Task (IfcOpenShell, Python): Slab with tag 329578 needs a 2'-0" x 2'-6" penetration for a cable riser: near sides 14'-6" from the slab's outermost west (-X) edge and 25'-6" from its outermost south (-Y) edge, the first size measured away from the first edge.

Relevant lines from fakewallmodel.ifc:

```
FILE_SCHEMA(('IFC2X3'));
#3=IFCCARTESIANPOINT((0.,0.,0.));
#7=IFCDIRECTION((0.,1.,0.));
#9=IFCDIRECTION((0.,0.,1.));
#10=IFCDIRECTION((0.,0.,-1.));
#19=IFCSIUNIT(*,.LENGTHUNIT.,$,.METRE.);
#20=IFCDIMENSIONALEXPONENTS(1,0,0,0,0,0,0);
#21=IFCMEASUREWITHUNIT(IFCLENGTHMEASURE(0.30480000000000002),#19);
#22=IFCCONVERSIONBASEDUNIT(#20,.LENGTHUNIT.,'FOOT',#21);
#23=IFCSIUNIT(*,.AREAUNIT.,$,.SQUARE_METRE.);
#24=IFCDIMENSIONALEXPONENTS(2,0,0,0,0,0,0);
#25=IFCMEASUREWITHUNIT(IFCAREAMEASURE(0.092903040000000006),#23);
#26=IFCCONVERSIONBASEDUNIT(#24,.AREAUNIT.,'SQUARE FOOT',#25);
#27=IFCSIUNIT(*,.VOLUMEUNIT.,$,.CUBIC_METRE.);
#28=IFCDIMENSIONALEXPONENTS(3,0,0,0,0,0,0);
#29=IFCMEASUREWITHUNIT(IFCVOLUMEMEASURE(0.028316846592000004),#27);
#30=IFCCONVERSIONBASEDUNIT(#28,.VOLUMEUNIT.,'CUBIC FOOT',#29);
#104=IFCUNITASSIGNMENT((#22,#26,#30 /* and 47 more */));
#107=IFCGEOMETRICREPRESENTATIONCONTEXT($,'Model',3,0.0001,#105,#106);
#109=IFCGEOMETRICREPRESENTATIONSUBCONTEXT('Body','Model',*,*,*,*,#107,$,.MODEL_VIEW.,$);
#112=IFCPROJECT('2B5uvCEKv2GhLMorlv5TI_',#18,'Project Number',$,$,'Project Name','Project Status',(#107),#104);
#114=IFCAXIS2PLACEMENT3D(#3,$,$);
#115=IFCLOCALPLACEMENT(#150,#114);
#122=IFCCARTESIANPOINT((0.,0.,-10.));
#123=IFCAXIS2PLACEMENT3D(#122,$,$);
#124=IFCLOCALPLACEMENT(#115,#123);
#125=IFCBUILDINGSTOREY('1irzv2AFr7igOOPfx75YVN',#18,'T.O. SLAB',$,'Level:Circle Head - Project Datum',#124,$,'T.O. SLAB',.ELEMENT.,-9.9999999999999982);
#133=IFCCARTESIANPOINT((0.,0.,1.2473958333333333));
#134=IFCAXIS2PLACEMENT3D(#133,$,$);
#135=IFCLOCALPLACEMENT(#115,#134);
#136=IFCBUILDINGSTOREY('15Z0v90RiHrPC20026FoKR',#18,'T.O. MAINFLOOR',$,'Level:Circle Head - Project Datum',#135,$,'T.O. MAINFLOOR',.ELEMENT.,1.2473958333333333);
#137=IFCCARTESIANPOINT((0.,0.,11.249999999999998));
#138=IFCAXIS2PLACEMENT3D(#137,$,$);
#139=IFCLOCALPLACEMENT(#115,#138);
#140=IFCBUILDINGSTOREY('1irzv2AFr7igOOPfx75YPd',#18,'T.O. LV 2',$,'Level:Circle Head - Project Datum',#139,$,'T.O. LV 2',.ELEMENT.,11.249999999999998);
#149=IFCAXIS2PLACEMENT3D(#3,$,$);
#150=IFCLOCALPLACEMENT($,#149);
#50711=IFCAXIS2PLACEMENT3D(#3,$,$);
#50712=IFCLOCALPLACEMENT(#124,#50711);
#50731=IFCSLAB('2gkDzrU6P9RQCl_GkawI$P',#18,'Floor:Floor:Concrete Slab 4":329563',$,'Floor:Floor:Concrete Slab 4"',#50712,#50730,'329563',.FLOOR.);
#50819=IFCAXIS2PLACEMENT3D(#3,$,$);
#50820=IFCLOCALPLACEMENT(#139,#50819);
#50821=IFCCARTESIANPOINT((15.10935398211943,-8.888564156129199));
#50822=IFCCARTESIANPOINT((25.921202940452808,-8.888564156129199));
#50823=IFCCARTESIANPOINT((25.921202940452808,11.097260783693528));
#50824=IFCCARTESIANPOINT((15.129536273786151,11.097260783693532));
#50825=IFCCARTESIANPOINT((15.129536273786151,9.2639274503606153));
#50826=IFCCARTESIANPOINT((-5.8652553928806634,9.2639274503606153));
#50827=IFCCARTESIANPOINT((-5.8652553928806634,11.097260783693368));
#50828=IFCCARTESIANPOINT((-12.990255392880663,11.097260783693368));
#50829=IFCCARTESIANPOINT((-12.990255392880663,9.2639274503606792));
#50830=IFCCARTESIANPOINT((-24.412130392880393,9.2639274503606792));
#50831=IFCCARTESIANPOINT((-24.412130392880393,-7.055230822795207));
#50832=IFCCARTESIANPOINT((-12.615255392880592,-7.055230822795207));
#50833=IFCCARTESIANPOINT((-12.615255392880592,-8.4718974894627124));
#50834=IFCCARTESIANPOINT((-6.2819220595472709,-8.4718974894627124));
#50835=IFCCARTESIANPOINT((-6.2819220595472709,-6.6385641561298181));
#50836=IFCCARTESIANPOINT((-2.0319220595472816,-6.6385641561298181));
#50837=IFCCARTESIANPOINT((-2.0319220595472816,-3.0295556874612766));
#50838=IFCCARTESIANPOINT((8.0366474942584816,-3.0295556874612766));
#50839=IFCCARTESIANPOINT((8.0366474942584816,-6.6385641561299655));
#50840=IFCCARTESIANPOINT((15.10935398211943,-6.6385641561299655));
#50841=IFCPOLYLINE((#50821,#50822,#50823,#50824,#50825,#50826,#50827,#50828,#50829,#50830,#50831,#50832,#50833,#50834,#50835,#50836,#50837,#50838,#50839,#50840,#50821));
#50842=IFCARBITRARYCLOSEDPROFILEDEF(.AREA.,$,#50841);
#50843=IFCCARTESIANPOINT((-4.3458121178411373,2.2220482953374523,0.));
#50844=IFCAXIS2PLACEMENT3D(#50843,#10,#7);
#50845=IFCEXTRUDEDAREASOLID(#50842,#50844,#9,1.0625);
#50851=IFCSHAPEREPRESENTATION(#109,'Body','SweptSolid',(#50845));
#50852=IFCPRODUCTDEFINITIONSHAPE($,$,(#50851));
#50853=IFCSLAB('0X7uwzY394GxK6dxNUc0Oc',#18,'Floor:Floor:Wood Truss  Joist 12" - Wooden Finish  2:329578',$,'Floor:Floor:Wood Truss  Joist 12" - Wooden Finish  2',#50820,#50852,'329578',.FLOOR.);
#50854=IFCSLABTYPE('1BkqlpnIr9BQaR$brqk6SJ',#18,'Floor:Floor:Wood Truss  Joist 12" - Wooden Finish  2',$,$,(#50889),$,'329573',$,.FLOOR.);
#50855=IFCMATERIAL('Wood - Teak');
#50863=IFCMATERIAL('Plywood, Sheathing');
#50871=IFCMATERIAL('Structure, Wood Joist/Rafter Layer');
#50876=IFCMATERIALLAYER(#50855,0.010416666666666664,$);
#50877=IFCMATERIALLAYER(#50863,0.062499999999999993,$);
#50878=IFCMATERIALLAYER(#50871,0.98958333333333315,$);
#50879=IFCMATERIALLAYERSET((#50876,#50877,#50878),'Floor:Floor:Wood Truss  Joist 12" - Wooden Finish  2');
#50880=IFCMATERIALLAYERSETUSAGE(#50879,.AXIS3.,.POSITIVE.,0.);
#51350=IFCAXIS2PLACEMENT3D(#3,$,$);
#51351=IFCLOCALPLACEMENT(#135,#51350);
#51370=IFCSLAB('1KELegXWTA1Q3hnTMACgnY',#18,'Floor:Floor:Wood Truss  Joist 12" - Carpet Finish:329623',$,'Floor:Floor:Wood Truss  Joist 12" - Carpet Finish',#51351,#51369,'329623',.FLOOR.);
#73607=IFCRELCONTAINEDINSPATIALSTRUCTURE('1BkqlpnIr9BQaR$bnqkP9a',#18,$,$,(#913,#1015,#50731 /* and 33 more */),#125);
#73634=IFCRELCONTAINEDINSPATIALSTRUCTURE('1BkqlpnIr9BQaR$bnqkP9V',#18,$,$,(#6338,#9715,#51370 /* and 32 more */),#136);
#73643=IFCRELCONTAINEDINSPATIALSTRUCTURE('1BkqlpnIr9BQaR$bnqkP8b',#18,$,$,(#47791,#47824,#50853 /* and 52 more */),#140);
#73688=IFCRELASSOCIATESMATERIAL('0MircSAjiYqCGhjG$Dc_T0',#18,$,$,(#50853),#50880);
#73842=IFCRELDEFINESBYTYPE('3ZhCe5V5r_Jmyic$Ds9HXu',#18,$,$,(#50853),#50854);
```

```python
import numpy as np
import ifcopenshell
import ifcopenshell.api.feature
import ifcopenshell.api.geometry
import ifcopenshell.api.root
import ifcopenshell.geom
import ifcopenshell.util.placement
import ifcopenshell.util.representation
import ifcopenshell.util.shape
import ifcopenshell.util.unit

model = ifcopenshell.open("fakewallmodel.ifc")
unit_scale = ifcopenshell.util.unit.calculate_unit_scale(model)
settings = ifcopenshell.geom.settings()


def volume(element):
    """Net volume in cubic metres, openings subtracted."""
    shape = ifcopenshell.geom.create_shape(settings, element)
    return ifcopenshell.util.shape.get_volume(shape.geometry)


slab = model.by_guid("0X7uwzY394GxK6dxNUc0Oc")
before = volume(slab)

# Extent in the slab's own axes, in metres. The edges named are its -X and -Y sides.
slab_shape = ifcopenshell.geom.create_shape(settings, slab)
vertices = ifcopenshell.util.shape.get_vertices(slab_shape.geometry)
x_min, y_min, bottom = vertices.min(axis=0)
top = vertices[:, 2].max()

opening = ifcopenshell.api.root.create_entity(model, ifc_class="IfcOpeningElement", name="Cable riser opening")
context = ifcopenshell.util.representation.get_context(model, "Model", "Body", "MODEL_VIEW")
width, depth = 0.6096, 0.762
outline = [(0.0, 0.0), (width, 0.0), (width, depth), (0.0, depth), (0.0, 0.0)]
# Overshoot both faces by 50 mm so the cut is clean.
shape = ifcopenshell.api.geometry.add_slab_representation(
    model, context=context, depth=top - bottom + 0.1, polyline=outline
)
ifcopenshell.api.geometry.assign_representation(model, product=opening, representation=shape)

matrix = ifcopenshell.util.placement.get_local_placement(slab.ObjectPlacement)
matrix[:, 3] = matrix @ np.append(np.array([x_min + 4.4196, y_min + 7.7724, bottom - 0.05]) / unit_scale, 1.0)
ifcopenshell.api.geometry.edit_object_placement(model, product=opening, matrix=matrix, is_si=False)
ifcopenshell.api.feature.add_feature(model, feature=opening, element=slab)

after = volume(slab)

print(f"slab volume {before:.3f} -> {after:.3f} m3")

model.write("fakewallmodel_v2.ifc")
```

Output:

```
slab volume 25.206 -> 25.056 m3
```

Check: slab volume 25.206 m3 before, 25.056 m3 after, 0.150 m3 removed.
